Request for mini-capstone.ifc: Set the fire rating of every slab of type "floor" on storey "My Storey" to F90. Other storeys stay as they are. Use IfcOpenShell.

First a look at what the model holds.

```python
import ifcopenshell
import ifcopenshell.util.element

model = ifcopenshell.open("mini-capstone.ifc")
print(model.schema)
storey = next(s for s in model.by_type("IfcBuildingStorey") if s.Name == "My Storey")
slabs = [e for e in ifcopenshell.util.element.get_decomposition(storey) if e.is_a("IfcSlab")]
seen = {}
for e in slabs:
    element_type = ifcopenshell.util.element.get_type(e)
    key = (element_type.Name if element_type != e and element_type else None, ifcopenshell.util.element.get_pset(e, "Pset_SlabCommon", "FireRating"))
    seen[key] = seen.get(key, 0) + 1
for (name, value), count in sorted(seen.items(), key=str):
    print(count, "x", name, "|", value)
```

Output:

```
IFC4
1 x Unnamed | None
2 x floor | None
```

```python
import ifcopenshell
import ifcopenshell.api.pset
import ifcopenshell.util.element

model = ifcopenshell.open("mini-capstone.ifc")

storey = next(s for s in model.by_type("IfcBuildingStorey") if s.Name == "My Storey")
slabs = [e for e in ifcopenshell.util.element.get_decomposition(storey) if e.is_a("IfcSlab")]

count = 0
for e in slabs:
    element_type = ifcopenshell.util.element.get_type(e)
    if element_type in (None, e) or element_type.Name != "floor":
        continue
    # add_pset returns the element's existing set when there is one.
    pset = ifcopenshell.api.pset.add_pset(model, product=e, name="Pset_SlabCommon")
    ifcopenshell.api.pset.edit_pset(model, pset=pset, properties={"FireRating": "F90"})
    count += 1

print(count, "slabs updated")

model.write("mini-capstone-out.ifc")
```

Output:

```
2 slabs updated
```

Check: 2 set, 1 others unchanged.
